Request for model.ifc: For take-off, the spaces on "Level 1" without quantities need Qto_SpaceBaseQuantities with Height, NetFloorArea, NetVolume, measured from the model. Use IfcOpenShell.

First a look at what the model holds.

```python
import ifcopenshell
import ifcopenshell.util.element
import ifcopenshell.util.unit

model = ifcopenshell.open("model.ifc")
print(model.schema)
for unit_type in ("LENGTHUNIT", "AREAUNIT", "VOLUMEUNIT"):
    print(unit_type, ifcopenshell.util.unit.calculate_unit_scale(model, unit_type))
storey = next(s for s in model.by_type("IfcBuildingStorey") if s.Name == "Level 1")
spaces = [e for e in ifcopenshell.util.element.get_decomposition(storey) if e.is_a("IfcSpace")]
for e in sorted(spaces, key=lambda e: e.id()):
    print(e.id(), e.is_a(), e.Name, list(ifcopenshell.util.element.get_psets(e, qtos_only=True)), sep=" | ")
```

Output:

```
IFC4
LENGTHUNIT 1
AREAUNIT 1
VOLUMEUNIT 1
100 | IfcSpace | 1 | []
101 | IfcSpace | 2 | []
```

```python
import ifcopenshell
import ifcopenshell.api.pset
import ifcopenshell.geom
import ifcopenshell.util.element
import ifcopenshell.util.shape
import ifcopenshell.util.unit

model = ifcopenshell.open("model.ifc")
unit_scale = ifcopenshell.util.unit.calculate_unit_scale(model)
area_scale = ifcopenshell.util.unit.calculate_unit_scale(model, "AREAUNIT")
volume_scale = ifcopenshell.util.unit.calculate_unit_scale(model, "VOLUMEUNIT")
settings = ifcopenshell.geom.settings()

storey = next(s for s in model.by_type("IfcBuildingStorey") if s.Name == "Level 1")
spaces = [e for e in ifcopenshell.util.element.get_decomposition(storey) if e.is_a("IfcSpace")]

for e in sorted(spaces, key=lambda e: e.id()):
    if ifcopenshell.util.element.get_psets(e, qtos_only=True, should_inherit=False):
        continue
    # Geometry comes back in metres, in the element's own axes.
    shape = ifcopenshell.geom.create_shape(settings, e)
    values = {
        "Height": ifcopenshell.util.shape.get_z(shape.geometry) / unit_scale,
        "NetFloorArea": ifcopenshell.util.shape.get_footprint_area(shape.geometry) / area_scale,
        "NetVolume": ifcopenshell.util.shape.get_volume(shape.geometry) / volume_scale,
    }
    qto = ifcopenshell.api.pset.add_qto(model, product=e, name="Qto_SpaceBaseQuantities")
    ifcopenshell.api.pset.edit_qto(model, qto=qto, properties=values)
    print(e.id(), {k: round(v, 3) for k, v in values.items()})

model.write("model_rev.ifc")
```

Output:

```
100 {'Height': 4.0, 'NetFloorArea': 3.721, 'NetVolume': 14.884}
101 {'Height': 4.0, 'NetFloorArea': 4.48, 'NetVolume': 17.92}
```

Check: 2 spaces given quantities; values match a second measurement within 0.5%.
